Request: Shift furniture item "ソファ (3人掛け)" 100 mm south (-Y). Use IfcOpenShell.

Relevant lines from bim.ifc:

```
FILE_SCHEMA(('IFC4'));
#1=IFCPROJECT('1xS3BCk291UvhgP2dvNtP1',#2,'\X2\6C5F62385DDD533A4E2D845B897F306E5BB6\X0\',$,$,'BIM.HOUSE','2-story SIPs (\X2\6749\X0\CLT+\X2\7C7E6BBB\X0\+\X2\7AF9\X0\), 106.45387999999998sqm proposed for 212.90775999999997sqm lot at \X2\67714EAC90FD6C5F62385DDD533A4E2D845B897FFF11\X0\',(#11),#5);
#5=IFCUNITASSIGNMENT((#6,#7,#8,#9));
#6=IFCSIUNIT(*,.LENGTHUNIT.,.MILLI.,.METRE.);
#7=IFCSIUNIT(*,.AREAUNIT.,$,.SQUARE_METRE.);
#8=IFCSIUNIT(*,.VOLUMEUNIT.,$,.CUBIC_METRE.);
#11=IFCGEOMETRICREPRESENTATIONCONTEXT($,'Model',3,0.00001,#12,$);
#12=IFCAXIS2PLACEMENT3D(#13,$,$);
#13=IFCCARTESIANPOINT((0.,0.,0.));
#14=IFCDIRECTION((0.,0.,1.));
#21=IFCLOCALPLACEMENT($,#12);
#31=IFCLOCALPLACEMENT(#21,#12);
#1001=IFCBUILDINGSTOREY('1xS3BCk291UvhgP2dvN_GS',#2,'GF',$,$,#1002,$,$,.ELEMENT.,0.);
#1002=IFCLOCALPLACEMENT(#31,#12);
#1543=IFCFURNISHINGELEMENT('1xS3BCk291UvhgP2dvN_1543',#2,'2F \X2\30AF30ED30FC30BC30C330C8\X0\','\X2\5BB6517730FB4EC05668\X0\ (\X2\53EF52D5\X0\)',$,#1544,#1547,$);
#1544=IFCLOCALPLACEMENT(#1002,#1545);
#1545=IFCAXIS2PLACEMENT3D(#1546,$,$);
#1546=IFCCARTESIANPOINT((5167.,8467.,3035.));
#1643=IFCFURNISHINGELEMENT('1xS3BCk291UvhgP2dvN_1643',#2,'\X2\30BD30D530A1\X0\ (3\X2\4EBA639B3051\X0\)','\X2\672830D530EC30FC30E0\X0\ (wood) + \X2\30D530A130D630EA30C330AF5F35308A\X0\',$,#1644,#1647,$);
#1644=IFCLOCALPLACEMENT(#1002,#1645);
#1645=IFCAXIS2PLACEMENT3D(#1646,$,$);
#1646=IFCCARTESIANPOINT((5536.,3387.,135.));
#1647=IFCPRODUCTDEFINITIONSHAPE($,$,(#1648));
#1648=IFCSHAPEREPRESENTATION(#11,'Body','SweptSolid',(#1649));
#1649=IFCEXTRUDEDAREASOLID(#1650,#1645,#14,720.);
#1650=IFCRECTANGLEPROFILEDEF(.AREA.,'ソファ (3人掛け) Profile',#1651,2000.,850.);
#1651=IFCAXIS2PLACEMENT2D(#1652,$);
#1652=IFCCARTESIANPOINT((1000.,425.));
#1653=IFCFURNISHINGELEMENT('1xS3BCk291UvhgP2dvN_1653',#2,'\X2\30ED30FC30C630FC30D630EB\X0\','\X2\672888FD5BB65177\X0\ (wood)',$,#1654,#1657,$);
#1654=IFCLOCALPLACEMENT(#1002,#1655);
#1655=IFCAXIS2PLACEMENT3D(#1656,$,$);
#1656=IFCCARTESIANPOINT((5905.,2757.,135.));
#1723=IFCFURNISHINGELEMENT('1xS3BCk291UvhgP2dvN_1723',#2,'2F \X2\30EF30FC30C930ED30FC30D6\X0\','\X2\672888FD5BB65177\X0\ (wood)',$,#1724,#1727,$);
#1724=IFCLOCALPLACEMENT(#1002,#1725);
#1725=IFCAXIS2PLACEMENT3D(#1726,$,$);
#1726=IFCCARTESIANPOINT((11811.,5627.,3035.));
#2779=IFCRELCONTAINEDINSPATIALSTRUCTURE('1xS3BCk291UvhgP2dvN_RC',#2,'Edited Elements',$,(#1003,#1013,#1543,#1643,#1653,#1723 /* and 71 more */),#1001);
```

```python
import ifcopenshell
import ifcopenshell.api.geometry
import ifcopenshell.util.placement
import ifcopenshell.util.unit

model = ifcopenshell.open("bim.ifc")
unit_scale = ifcopenshell.util.unit.calculate_unit_scale(model)

item = model.by_id(1643)
matrix = ifcopenshell.util.placement.get_local_placement(item.ObjectPlacement)
matrix[1, 3] -= 0.1 / unit_scale
ifcopenshell.api.geometry.edit_object_placement(model, product=item, matrix=matrix, is_si=False)

print(ifcopenshell.util.placement.get_local_placement(item.ObjectPlacement).round(3) + 0.0)

model.write("bim_updated.ifc")
```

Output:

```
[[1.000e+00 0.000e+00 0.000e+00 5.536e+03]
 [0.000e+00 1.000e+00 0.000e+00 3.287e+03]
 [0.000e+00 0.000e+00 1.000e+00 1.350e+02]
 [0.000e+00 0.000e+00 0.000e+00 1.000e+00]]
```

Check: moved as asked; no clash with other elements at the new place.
